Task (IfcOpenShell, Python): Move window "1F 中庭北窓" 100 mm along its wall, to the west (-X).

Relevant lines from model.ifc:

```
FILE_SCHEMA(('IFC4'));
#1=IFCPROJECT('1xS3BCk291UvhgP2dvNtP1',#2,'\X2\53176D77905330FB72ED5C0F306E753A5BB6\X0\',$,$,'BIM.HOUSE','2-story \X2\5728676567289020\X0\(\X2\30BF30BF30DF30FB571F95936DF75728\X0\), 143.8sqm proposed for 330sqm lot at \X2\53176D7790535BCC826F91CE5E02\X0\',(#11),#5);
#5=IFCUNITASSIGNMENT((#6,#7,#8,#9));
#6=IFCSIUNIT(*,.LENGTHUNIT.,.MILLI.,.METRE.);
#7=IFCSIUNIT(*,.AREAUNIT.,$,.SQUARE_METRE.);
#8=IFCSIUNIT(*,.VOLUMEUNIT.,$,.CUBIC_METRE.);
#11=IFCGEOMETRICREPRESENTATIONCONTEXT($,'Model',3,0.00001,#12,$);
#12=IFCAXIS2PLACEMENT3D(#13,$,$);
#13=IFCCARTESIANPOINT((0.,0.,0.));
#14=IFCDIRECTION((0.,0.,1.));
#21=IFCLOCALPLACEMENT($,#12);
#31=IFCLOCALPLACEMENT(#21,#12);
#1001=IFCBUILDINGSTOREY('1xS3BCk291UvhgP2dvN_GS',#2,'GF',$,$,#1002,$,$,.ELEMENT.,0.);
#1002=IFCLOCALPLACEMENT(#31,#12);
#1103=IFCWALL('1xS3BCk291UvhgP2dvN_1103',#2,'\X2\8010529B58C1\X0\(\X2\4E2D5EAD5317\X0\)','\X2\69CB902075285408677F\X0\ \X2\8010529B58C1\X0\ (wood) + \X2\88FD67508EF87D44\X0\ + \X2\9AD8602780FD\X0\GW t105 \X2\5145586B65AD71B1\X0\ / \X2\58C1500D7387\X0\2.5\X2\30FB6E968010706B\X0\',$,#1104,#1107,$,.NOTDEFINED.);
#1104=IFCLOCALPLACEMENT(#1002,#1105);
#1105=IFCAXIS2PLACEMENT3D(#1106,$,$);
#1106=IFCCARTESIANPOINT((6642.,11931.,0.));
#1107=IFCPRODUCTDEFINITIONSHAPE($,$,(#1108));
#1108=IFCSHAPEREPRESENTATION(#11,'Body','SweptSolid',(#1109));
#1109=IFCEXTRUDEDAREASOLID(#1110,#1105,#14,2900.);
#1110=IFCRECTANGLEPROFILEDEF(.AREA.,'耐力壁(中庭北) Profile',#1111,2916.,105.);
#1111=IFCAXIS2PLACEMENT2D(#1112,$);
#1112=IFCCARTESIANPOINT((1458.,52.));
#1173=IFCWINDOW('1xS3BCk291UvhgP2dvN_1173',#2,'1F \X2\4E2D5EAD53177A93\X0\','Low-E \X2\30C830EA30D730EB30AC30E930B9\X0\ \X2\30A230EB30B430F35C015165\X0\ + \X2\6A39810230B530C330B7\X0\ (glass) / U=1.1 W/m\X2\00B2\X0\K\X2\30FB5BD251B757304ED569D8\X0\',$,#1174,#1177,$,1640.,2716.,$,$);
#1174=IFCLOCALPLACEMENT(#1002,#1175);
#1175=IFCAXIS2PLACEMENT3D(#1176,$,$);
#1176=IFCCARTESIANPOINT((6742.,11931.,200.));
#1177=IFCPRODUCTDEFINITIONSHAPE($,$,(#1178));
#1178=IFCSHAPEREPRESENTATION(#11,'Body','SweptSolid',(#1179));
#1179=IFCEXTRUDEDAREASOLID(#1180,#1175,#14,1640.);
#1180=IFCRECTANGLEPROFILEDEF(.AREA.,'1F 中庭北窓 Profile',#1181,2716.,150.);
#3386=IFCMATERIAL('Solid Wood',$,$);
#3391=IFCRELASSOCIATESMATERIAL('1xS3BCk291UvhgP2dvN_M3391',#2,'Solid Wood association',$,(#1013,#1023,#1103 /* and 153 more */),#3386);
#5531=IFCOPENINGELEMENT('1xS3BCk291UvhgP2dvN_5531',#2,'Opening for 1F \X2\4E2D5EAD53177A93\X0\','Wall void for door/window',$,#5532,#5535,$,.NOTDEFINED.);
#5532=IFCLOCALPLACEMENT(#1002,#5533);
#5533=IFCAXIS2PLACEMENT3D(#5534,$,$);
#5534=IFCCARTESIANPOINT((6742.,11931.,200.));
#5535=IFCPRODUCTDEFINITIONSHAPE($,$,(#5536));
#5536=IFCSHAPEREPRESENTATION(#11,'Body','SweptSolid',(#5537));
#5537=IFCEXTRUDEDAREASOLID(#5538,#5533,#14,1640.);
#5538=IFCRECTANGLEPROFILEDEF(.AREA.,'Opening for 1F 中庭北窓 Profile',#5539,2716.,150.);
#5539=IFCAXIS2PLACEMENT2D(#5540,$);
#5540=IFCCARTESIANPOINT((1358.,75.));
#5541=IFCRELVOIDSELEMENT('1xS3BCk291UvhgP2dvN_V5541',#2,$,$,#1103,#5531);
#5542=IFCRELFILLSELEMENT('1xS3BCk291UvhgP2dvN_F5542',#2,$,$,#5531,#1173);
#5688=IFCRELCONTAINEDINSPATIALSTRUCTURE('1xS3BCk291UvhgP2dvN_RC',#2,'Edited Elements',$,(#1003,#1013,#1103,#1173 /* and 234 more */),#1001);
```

```python
import ifcopenshell
import ifcopenshell.api.geometry
import ifcopenshell.util.placement
import ifcopenshell.util.unit

model = ifcopenshell.open("model.ifc")
unit_scale = ifcopenshell.util.unit.calculate_unit_scale(model)

window = model.by_guid("1xS3BCk291UvhgP2dvN_1173")
opening = window.FillsVoids[0].RelatingOpeningElement
wall = opening.VoidsElements[0].RelatingBuildingElement

wall_matrix = ifcopenshell.util.placement.get_local_placement(wall.ObjectPlacement)
shift = wall_matrix[:3, 0] * -0.1 / unit_scale
before = ifcopenshell.util.placement.get_local_placement(window.ObjectPlacement)[:3, 3].copy()

# The window is not placed relative to its opening, so move both.
for product in (opening, window):
    matrix = ifcopenshell.util.placement.get_local_placement(product.ObjectPlacement)
    matrix[:3, 3] += shift
    ifcopenshell.api.geometry.edit_object_placement(model, product=product, matrix=matrix, is_si=False)

after = ifcopenshell.util.placement.get_local_placement(window.ObjectPlacement)[:3, 3]
print("window moved by", (after - before).round(3) + 0.0)

model.write("model_edited.ifc")
```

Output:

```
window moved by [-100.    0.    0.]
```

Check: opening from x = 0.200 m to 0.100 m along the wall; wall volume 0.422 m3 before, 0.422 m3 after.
